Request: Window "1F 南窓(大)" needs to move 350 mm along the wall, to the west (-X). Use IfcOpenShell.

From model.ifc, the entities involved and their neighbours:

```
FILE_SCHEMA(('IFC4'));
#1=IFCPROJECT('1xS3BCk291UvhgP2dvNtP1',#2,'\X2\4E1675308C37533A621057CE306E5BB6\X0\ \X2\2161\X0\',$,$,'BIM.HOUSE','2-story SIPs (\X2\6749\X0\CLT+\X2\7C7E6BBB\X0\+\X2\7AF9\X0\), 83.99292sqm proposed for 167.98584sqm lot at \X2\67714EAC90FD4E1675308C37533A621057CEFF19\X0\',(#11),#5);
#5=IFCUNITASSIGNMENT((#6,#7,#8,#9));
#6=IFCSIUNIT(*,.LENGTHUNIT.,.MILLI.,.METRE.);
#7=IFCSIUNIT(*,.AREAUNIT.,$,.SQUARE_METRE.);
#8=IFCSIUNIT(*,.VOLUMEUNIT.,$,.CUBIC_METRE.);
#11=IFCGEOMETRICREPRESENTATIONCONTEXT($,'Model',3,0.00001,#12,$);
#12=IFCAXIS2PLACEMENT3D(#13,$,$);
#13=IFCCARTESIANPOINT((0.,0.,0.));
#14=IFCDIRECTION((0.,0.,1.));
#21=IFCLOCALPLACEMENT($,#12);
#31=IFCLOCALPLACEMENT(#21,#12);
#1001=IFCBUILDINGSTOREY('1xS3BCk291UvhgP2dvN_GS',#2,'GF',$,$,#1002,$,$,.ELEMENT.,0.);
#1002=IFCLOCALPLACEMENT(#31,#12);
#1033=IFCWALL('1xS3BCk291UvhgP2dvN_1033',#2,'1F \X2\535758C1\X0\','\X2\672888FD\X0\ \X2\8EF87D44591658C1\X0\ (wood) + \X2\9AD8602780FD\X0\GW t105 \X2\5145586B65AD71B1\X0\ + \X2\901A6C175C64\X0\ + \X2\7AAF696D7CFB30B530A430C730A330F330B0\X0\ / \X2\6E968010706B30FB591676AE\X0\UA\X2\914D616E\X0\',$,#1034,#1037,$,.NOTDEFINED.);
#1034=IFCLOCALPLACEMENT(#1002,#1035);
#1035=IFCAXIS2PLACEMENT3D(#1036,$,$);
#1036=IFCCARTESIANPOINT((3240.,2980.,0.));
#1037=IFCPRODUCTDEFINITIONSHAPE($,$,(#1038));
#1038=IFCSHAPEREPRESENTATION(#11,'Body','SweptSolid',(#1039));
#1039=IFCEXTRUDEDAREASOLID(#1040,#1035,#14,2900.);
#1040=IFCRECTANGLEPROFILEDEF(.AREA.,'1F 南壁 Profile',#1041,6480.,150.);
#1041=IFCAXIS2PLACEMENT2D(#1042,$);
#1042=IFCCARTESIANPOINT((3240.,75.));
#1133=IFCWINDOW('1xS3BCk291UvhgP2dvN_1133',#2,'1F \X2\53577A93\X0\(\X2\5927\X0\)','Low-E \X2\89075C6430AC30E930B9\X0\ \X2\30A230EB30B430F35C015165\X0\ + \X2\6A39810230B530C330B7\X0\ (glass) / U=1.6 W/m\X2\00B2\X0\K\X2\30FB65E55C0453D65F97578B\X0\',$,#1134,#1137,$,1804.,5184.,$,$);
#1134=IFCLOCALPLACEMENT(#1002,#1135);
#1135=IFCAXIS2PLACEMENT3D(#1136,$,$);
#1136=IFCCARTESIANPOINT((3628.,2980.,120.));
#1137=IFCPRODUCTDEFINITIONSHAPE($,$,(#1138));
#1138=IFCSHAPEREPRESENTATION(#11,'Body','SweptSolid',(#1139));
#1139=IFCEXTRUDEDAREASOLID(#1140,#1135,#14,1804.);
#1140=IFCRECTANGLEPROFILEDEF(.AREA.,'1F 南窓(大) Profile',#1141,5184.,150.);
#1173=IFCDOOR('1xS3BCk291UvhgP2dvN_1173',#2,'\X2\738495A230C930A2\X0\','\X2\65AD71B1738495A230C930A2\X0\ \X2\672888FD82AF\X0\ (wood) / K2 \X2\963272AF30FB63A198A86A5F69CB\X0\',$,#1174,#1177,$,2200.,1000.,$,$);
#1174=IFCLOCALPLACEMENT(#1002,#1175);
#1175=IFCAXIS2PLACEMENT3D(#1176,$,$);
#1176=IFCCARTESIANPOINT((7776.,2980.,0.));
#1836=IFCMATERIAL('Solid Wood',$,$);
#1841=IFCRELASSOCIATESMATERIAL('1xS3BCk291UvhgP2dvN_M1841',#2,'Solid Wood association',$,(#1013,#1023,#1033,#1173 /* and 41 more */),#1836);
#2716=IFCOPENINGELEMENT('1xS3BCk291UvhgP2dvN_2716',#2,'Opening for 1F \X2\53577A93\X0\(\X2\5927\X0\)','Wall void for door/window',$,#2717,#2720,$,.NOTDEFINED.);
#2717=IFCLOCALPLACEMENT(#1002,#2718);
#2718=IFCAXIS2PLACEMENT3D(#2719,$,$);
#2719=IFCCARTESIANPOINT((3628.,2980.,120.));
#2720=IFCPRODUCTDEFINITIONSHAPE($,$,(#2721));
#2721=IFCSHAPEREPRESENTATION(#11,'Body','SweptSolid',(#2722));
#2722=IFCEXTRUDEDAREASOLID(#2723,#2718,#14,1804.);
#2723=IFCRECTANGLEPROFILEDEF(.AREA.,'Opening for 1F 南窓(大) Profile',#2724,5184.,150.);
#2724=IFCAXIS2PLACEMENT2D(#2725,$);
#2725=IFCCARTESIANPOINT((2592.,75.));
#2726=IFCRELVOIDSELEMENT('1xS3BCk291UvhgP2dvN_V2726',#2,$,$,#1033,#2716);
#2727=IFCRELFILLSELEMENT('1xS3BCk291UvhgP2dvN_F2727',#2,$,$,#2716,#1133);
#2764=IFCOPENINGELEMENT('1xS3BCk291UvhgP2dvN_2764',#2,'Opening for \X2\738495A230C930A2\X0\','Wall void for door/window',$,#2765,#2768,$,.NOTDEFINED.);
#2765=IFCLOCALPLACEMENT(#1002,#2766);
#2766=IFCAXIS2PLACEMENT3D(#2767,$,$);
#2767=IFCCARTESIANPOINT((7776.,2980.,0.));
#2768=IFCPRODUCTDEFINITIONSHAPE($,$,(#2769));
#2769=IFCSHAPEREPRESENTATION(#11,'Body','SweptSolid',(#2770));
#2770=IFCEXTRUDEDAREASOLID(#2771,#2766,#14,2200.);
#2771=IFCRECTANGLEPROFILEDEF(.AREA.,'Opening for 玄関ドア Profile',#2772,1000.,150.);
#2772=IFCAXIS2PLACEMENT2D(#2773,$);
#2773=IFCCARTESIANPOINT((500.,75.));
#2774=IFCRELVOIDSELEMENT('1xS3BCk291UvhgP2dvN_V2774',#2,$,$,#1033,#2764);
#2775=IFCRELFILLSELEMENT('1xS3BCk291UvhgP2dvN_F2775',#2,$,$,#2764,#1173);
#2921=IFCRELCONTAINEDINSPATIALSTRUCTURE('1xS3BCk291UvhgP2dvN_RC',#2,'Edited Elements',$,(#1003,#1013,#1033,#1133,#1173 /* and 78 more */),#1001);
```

```python
import ifcopenshell
import ifcopenshell.api.geometry
import ifcopenshell.util.placement

model = ifcopenshell.open("model.ifc")

window = model.by_id(1133)
opening = window.FillsVoids[0].RelatingOpeningElement
wall = opening.VoidsElements[0].RelatingBuildingElement

wall_matrix = ifcopenshell.util.placement.get_local_placement(wall.ObjectPlacement)
shift = wall_matrix[:3, 0] * -350.0
before = ifcopenshell.util.placement.get_local_placement(window.ObjectPlacement)[:3, 3].copy()

# The window is not placed relative to its opening, so move both.
for product in (opening, window):
    matrix = ifcopenshell.util.placement.get_local_placement(product.ObjectPlacement)
    matrix[:3, 3] += shift
    ifcopenshell.api.geometry.edit_object_placement(model, product=product, matrix=matrix, is_si=False)

after = ifcopenshell.util.placement.get_local_placement(window.ObjectPlacement)[:3, 3]
print("window moved by", (after - before).round(3) + 0.0)

model.write("model_rev.ifc")
```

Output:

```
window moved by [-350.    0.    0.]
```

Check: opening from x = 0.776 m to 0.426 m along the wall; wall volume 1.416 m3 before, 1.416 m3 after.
